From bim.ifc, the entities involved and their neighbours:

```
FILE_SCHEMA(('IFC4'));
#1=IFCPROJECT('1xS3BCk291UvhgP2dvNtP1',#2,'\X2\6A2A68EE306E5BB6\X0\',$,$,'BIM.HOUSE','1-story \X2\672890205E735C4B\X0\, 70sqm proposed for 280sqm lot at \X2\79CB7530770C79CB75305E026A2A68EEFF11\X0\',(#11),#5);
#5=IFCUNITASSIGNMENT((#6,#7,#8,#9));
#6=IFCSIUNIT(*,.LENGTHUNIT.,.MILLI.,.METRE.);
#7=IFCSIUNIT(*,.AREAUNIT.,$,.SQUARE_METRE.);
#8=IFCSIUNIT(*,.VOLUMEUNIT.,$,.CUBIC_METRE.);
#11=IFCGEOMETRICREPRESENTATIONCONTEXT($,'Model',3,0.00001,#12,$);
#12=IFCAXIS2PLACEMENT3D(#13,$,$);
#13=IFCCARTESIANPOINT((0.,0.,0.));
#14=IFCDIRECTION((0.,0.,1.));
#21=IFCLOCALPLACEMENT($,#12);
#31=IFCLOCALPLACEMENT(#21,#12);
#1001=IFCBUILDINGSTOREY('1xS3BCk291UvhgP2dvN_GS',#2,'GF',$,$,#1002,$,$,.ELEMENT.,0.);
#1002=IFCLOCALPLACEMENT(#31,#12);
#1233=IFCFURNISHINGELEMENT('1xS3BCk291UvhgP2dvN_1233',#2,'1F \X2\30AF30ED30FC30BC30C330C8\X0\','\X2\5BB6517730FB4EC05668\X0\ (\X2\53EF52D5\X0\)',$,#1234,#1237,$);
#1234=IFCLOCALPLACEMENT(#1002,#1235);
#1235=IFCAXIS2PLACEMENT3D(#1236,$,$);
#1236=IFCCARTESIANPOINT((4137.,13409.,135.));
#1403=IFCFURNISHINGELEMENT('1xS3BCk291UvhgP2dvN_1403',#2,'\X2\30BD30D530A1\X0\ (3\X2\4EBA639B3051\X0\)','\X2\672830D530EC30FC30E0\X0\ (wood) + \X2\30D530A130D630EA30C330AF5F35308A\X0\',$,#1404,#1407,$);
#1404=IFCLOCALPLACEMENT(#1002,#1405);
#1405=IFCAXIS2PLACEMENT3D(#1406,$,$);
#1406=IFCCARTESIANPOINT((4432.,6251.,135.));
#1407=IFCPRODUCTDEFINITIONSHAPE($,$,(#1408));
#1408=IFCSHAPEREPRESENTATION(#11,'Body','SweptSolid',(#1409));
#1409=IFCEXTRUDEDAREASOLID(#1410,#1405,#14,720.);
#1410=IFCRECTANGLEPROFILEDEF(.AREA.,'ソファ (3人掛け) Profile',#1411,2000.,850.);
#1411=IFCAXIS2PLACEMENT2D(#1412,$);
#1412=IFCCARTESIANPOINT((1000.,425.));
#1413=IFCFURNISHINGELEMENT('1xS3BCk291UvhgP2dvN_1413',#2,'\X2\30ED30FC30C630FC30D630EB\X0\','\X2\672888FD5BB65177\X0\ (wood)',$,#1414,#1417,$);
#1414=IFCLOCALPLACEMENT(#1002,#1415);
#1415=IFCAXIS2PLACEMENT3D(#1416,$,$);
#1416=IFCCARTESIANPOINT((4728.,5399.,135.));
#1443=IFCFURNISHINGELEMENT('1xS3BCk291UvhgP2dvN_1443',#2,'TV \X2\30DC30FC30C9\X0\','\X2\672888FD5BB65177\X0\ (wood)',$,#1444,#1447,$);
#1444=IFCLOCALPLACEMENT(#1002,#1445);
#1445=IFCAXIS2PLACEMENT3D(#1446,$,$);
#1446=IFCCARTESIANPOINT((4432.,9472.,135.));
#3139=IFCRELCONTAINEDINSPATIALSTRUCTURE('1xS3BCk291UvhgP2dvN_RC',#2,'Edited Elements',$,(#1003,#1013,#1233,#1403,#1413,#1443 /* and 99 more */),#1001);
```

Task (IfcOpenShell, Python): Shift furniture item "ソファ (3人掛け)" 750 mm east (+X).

```python
import ifcopenshell
import ifcopenshell.api.geometry
import ifcopenshell.util.placement

model = ifcopenshell.open("bim.ifc")

item = model.by_guid("1xS3BCk291UvhgP2dvN_1403")
matrix = ifcopenshell.util.placement.get_local_placement(item.ObjectPlacement)
matrix[0, 3] += 750.0
ifcopenshell.api.geometry.edit_object_placement(model, product=item, matrix=matrix, is_si=False)

print(ifcopenshell.util.placement.get_local_placement(item.ObjectPlacement).round(3) + 0.0)

model.write("bim_updated.ifc")
```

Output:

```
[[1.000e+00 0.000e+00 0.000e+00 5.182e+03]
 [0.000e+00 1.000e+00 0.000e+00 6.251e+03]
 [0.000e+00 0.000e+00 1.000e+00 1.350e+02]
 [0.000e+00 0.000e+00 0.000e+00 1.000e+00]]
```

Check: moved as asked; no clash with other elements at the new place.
